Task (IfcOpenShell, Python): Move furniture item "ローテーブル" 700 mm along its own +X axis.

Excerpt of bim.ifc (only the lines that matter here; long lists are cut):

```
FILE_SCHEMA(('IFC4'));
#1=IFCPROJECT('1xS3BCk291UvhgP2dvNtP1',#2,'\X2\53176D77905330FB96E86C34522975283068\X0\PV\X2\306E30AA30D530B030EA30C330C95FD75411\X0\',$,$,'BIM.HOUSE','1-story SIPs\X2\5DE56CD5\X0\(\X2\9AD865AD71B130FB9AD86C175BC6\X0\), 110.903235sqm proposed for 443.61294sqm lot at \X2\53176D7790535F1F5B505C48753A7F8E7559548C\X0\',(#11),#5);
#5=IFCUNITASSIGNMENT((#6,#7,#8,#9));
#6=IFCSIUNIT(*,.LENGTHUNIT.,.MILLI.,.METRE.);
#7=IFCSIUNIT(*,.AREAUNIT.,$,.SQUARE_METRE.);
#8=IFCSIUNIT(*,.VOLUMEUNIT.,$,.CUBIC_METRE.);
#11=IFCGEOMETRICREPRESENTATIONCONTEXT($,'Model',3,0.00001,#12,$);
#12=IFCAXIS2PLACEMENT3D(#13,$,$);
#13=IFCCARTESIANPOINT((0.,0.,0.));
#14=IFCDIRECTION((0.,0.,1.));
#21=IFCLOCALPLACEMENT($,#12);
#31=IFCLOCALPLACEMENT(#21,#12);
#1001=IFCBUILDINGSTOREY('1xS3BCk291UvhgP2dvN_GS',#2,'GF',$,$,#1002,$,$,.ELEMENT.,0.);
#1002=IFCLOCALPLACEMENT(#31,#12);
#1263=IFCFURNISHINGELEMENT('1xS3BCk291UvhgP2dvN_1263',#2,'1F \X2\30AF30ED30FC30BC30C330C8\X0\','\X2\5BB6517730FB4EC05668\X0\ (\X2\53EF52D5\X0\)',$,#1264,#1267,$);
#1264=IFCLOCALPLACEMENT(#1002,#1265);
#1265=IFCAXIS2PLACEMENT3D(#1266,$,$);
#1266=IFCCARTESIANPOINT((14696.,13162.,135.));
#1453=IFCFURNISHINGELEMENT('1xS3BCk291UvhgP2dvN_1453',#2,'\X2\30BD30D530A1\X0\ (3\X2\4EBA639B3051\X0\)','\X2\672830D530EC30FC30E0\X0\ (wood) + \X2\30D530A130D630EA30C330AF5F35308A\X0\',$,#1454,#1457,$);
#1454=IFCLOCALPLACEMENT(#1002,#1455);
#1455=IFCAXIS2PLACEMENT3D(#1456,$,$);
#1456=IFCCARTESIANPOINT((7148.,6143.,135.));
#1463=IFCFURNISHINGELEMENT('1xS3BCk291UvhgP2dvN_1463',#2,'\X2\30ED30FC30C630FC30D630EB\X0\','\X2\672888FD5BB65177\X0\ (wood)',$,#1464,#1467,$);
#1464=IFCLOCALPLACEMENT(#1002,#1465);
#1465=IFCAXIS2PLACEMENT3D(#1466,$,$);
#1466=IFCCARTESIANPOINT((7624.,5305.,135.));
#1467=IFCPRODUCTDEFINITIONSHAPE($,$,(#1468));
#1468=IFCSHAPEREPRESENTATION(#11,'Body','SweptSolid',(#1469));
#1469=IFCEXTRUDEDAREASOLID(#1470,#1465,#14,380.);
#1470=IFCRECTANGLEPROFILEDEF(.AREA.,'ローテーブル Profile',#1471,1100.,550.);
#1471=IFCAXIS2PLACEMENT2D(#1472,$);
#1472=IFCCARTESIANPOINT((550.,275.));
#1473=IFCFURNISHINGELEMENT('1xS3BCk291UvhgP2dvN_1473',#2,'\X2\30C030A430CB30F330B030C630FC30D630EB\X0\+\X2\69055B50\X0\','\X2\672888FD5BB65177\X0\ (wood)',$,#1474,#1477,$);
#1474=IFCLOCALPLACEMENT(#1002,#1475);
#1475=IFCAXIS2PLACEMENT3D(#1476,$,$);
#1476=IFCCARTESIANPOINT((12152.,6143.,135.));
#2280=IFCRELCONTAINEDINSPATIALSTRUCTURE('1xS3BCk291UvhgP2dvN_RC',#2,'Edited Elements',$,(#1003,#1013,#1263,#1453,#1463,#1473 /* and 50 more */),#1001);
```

```python
import ifcopenshell
import ifcopenshell.api.geometry
import ifcopenshell.util.placement
import ifcopenshell.util.unit

model = ifcopenshell.open("bim.ifc")
unit_scale = ifcopenshell.util.unit.calculate_unit_scale(model)

item = model.by_id(1463)
matrix = ifcopenshell.util.placement.get_local_placement(item.ObjectPlacement)
matrix[:3, 3] += matrix[:3, 0] * 0.7 / unit_scale
ifcopenshell.api.geometry.edit_object_placement(model, product=item, matrix=matrix, is_si=False)

print(ifcopenshell.util.placement.get_local_placement(item.ObjectPlacement).round(3) + 0.0)

model.write("bim-out.ifc")
```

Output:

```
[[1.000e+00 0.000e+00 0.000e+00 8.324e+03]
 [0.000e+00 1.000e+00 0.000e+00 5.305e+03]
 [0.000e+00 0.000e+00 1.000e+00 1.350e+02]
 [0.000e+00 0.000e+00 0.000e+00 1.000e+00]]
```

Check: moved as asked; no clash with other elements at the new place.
